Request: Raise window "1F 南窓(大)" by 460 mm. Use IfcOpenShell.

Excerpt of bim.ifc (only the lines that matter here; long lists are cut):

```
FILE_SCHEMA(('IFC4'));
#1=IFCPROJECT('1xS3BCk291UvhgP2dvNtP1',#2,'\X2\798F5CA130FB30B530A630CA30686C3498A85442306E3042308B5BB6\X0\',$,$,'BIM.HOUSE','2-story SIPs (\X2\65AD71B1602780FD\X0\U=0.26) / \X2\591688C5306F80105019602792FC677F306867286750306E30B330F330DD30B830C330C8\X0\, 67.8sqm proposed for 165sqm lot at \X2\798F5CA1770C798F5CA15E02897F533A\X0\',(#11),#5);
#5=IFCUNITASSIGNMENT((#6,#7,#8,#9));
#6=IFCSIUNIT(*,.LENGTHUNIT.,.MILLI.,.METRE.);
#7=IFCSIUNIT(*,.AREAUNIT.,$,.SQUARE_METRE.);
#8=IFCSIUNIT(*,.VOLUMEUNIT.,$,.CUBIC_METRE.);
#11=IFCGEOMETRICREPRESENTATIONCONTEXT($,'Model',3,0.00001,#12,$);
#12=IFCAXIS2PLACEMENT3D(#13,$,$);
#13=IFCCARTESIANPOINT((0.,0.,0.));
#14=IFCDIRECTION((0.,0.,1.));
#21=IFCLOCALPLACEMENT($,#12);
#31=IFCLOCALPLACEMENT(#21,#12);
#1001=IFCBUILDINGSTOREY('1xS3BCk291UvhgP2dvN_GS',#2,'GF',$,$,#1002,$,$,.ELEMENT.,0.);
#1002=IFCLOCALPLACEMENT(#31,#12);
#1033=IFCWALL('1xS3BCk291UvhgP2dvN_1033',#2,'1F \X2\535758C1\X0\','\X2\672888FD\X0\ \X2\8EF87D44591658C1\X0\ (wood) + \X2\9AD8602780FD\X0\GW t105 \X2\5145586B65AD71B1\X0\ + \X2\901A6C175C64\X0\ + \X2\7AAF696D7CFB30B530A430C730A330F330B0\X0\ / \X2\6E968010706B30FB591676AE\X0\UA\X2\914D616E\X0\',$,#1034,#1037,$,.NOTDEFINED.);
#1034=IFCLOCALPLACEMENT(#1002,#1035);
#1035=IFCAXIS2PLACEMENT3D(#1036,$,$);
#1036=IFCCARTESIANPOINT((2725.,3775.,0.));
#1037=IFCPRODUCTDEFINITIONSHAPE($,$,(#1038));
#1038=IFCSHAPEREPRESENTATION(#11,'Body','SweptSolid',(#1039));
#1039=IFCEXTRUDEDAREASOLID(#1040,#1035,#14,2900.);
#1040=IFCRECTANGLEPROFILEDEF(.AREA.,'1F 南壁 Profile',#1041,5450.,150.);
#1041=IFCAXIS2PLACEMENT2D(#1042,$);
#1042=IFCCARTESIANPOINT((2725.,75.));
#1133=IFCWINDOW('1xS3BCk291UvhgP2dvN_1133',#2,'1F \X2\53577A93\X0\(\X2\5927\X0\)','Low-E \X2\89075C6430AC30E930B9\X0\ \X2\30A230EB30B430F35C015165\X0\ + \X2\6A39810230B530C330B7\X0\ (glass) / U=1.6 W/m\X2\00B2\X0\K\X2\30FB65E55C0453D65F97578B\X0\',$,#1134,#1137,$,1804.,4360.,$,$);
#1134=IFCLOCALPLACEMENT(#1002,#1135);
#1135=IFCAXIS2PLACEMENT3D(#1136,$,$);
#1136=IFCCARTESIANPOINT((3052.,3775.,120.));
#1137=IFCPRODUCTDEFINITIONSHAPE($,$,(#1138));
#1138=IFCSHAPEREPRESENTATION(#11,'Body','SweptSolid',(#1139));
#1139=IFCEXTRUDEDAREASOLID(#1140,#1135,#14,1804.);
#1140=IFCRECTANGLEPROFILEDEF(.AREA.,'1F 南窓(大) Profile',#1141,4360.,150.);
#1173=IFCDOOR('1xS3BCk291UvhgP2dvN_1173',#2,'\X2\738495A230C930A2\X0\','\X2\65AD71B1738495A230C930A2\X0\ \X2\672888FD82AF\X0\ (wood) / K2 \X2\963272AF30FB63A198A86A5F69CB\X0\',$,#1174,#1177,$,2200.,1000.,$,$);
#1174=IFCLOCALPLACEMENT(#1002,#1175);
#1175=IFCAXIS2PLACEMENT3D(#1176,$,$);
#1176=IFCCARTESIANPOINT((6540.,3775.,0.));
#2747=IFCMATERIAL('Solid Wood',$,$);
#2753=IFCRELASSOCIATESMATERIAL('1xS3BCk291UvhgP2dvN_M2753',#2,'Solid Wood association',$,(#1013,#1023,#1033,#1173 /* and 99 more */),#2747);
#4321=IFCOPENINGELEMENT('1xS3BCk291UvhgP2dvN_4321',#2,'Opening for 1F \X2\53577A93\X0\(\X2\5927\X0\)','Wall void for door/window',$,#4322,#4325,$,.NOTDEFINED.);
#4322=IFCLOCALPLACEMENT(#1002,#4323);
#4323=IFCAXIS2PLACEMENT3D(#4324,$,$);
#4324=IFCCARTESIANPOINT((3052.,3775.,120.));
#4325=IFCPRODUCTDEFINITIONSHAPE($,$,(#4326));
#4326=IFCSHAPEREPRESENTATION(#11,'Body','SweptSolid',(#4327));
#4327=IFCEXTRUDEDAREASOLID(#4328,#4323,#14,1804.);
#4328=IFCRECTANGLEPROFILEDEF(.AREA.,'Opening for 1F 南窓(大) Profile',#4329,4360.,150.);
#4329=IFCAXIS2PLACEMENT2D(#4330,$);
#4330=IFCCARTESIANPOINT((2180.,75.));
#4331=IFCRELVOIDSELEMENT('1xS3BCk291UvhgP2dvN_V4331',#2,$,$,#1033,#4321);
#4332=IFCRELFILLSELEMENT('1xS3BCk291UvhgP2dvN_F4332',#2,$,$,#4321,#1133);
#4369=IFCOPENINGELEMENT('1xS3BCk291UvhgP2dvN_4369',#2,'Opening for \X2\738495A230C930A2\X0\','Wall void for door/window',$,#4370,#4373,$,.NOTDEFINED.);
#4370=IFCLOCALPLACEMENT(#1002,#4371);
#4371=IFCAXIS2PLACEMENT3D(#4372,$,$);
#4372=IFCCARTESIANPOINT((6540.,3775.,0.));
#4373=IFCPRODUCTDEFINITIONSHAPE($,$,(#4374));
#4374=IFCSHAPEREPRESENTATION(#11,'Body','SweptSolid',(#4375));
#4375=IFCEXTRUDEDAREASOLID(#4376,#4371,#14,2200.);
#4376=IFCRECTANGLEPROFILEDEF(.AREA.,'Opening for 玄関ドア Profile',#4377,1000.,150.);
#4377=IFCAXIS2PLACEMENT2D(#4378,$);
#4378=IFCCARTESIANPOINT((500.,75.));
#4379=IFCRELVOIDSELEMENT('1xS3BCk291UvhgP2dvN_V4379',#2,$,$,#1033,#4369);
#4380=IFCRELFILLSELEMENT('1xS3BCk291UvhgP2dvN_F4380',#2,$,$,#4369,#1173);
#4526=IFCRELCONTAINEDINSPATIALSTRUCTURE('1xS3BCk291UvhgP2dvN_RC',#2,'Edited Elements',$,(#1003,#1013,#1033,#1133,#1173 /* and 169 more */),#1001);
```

```python
import numpy as np
import ifcopenshell
import ifcopenshell.api.geometry
import ifcopenshell.util.placement
import ifcopenshell.util.unit

model = ifcopenshell.open("bim.ifc")
unit_scale = ifcopenshell.util.unit.calculate_unit_scale(model)

window = model.by_guid("1xS3BCk291UvhgP2dvN_1133")
opening = window.FillsVoids[0].RelatingOpeningElement
dz = 0.46 / unit_scale

shift = np.array([0.0, 0.0, dz])
# The window is not placed relative to its opening, so move both.
for product in (opening, window):
    matrix = ifcopenshell.util.placement.get_local_placement(product.ObjectPlacement)
    matrix[:3, 3] += shift
    ifcopenshell.api.geometry.edit_object_placement(model, product=product, matrix=matrix, is_si=False)

print(f"moved by {dz * unit_scale:+.3f} m")

model.write("bim-out.ifc")
```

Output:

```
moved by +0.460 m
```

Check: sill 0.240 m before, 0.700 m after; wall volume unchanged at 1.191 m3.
